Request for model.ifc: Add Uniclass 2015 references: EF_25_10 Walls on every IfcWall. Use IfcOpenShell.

First a look at what the model holds.

```python
import ifcopenshell

model = ifcopenshell.open("model.ifc")
print(model.schema)
print("classifications:", [c.Name for c in model.by_type("IfcClassification")])
for ifc_class in ("IfcDoor", "IfcRoof", "IfcStair", "IfcWall", "IfcWindow"):
    print(ifc_class, len(model.by_type(ifc_class)))
```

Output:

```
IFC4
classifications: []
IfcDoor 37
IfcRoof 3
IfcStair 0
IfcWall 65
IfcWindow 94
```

```python
import ifcopenshell
import ifcopenshell.api.classification

model = ifcopenshell.open("model.ifc")

system = ifcopenshell.api.classification.add_classification(model, classification="Uniclass 2015")

codes = {
    "IfcWall": ("EF_25_10", "Walls"),
}
for ifc_class, (code, name) in codes.items():
    products = model.by_type(ifc_class)
    ifcopenshell.api.classification.add_reference(
        model, products=products, classification=system, identification=code, name=name
    )
    print(code, len(products))

model.write("model_rev.ifc")
```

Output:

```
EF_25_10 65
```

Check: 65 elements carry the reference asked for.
